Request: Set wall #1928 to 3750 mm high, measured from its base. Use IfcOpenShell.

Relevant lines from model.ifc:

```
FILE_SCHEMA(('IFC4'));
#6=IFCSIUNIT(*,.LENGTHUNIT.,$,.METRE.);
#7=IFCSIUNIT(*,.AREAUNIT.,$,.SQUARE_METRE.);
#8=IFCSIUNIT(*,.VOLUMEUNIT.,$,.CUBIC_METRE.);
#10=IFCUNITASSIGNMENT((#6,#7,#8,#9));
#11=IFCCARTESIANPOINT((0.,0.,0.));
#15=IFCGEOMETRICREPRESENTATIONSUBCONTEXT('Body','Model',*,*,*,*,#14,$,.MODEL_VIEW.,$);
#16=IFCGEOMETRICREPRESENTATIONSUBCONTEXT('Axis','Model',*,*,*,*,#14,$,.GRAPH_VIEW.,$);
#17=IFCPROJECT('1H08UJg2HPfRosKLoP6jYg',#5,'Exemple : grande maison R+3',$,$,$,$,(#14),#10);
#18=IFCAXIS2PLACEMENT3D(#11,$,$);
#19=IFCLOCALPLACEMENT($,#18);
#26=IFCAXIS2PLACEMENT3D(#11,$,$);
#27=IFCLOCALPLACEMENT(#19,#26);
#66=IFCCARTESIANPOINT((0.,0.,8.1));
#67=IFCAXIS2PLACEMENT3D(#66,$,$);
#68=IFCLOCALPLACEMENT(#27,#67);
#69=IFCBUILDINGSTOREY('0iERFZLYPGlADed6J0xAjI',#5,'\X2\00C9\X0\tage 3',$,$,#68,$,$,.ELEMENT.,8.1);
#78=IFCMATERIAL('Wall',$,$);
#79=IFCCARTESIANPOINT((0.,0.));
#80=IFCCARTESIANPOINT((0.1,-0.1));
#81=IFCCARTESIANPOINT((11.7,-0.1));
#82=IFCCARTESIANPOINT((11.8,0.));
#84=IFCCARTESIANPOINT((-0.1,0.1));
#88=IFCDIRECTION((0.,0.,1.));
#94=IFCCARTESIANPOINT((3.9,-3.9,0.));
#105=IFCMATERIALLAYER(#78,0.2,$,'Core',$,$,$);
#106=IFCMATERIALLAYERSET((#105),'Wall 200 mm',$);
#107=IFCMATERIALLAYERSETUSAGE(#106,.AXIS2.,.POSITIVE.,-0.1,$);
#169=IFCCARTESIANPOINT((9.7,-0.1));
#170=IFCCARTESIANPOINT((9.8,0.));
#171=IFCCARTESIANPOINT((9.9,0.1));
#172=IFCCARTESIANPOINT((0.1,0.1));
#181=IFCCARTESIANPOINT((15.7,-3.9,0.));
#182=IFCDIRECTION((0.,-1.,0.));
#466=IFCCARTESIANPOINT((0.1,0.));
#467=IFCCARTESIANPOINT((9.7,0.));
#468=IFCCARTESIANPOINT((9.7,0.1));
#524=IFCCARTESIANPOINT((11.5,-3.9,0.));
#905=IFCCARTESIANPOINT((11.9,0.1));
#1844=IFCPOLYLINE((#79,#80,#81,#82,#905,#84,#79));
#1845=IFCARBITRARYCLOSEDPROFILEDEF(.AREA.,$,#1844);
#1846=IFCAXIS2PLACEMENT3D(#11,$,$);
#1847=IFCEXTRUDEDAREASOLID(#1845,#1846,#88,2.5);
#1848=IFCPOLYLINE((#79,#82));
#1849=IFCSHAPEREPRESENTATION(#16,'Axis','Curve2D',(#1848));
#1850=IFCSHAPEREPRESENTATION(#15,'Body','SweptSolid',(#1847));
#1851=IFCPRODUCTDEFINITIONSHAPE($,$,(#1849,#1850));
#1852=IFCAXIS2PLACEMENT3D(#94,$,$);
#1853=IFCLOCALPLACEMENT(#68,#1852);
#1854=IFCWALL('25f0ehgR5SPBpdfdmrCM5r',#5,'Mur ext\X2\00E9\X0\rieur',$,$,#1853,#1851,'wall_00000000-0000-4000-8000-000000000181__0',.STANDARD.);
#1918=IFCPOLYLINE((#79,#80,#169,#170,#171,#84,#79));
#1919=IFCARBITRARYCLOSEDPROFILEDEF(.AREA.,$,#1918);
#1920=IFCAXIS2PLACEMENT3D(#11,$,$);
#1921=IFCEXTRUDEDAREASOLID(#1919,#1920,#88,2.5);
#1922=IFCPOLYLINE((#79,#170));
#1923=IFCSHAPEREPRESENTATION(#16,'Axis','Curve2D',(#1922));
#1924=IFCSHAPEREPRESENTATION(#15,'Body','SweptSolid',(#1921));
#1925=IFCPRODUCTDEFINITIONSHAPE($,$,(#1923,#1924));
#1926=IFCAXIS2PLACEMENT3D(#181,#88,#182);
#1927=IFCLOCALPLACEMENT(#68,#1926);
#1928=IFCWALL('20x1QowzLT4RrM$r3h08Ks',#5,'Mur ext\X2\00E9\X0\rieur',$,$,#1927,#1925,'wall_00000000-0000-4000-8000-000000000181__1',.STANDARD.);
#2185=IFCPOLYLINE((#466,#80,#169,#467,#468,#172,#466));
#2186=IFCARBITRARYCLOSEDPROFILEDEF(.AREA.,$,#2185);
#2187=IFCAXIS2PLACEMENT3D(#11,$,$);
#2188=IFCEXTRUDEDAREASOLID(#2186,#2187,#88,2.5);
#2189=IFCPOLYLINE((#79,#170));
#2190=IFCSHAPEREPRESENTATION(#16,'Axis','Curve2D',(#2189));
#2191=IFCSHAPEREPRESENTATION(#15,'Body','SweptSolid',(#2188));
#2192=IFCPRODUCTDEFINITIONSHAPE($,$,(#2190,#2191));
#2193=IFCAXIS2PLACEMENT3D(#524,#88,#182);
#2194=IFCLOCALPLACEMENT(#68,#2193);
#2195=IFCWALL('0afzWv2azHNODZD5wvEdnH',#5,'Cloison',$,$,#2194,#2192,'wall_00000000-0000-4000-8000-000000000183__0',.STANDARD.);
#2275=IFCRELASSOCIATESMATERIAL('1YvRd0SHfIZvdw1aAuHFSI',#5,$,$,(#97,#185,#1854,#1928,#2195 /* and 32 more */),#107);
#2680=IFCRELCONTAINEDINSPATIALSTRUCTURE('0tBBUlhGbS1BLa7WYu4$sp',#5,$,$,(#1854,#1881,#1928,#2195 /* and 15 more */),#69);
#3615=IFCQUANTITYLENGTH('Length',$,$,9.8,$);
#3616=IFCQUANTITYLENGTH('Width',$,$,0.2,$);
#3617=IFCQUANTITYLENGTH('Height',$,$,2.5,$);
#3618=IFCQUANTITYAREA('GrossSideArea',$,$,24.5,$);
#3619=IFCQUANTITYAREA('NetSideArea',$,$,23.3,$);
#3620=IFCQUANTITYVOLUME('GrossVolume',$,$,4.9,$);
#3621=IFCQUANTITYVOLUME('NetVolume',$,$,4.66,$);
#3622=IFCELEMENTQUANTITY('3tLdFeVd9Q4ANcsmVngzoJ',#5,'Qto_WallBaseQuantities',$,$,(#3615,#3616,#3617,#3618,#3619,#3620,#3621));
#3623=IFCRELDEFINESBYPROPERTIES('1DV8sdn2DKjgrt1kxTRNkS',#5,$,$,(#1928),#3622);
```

```python
import ifcopenshell
import ifcopenshell.api.pset
import ifcopenshell.geom
import ifcopenshell.util.element
import ifcopenshell.util.representation
import ifcopenshell.util.shape
import ifcopenshell.util.unit

model = ifcopenshell.open("model.ifc")
unit_scale = ifcopenshell.util.unit.calculate_unit_scale(model)
area_scale = ifcopenshell.util.unit.calculate_unit_scale(model, "AREAUNIT")
volume_scale = ifcopenshell.util.unit.calculate_unit_scale(model, "VOLUMEUNIT")
settings = ifcopenshell.geom.settings()


def volume(element):
    """Net volume in cubic metres, openings subtracted."""
    shape = ifcopenshell.geom.create_shape(settings, element)
    return ifcopenshell.util.shape.get_volume(shape.geometry)


wall = model.by_id(1928)
before = volume(wall)

body = ifcopenshell.util.representation.get_representation(wall, "Model", "Body")
solid = body.Items[0]
old_height = solid.Depth
solid.Depth = 3.75 / unit_scale
after = volume(wall)
thickness = 0.2  # wall thickness in metres

# Update the stored height, areas and volumes.
qto = model.by_id(ifcopenshell.util.element.get_pset(wall, "Qto_WallBaseQuantities", should_inherit=False)["id"])
ifcopenshell.api.pset.edit_qto(model, qto=qto, properties={
    "Height": solid.Depth,
    "GrossSideArea": ifcopenshell.util.element.get_pset(wall, "Qto_WallBaseQuantities", "GrossSideArea") * solid.Depth / old_height,
    "NetSideArea": after / thickness / area_scale,
    "GrossVolume": ifcopenshell.util.element.get_pset(wall, "Qto_WallBaseQuantities", "GrossVolume") * solid.Depth / old_height,
    "NetVolume": after / volume_scale,
})

print(f"height {old_height:g} -> {solid.Depth:g}, volume {before:.3f} -> {after:.3f} m3")

model.write("model_rev.ifc")
```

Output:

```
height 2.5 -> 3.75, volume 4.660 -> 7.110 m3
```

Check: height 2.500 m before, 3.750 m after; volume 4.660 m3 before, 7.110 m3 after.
